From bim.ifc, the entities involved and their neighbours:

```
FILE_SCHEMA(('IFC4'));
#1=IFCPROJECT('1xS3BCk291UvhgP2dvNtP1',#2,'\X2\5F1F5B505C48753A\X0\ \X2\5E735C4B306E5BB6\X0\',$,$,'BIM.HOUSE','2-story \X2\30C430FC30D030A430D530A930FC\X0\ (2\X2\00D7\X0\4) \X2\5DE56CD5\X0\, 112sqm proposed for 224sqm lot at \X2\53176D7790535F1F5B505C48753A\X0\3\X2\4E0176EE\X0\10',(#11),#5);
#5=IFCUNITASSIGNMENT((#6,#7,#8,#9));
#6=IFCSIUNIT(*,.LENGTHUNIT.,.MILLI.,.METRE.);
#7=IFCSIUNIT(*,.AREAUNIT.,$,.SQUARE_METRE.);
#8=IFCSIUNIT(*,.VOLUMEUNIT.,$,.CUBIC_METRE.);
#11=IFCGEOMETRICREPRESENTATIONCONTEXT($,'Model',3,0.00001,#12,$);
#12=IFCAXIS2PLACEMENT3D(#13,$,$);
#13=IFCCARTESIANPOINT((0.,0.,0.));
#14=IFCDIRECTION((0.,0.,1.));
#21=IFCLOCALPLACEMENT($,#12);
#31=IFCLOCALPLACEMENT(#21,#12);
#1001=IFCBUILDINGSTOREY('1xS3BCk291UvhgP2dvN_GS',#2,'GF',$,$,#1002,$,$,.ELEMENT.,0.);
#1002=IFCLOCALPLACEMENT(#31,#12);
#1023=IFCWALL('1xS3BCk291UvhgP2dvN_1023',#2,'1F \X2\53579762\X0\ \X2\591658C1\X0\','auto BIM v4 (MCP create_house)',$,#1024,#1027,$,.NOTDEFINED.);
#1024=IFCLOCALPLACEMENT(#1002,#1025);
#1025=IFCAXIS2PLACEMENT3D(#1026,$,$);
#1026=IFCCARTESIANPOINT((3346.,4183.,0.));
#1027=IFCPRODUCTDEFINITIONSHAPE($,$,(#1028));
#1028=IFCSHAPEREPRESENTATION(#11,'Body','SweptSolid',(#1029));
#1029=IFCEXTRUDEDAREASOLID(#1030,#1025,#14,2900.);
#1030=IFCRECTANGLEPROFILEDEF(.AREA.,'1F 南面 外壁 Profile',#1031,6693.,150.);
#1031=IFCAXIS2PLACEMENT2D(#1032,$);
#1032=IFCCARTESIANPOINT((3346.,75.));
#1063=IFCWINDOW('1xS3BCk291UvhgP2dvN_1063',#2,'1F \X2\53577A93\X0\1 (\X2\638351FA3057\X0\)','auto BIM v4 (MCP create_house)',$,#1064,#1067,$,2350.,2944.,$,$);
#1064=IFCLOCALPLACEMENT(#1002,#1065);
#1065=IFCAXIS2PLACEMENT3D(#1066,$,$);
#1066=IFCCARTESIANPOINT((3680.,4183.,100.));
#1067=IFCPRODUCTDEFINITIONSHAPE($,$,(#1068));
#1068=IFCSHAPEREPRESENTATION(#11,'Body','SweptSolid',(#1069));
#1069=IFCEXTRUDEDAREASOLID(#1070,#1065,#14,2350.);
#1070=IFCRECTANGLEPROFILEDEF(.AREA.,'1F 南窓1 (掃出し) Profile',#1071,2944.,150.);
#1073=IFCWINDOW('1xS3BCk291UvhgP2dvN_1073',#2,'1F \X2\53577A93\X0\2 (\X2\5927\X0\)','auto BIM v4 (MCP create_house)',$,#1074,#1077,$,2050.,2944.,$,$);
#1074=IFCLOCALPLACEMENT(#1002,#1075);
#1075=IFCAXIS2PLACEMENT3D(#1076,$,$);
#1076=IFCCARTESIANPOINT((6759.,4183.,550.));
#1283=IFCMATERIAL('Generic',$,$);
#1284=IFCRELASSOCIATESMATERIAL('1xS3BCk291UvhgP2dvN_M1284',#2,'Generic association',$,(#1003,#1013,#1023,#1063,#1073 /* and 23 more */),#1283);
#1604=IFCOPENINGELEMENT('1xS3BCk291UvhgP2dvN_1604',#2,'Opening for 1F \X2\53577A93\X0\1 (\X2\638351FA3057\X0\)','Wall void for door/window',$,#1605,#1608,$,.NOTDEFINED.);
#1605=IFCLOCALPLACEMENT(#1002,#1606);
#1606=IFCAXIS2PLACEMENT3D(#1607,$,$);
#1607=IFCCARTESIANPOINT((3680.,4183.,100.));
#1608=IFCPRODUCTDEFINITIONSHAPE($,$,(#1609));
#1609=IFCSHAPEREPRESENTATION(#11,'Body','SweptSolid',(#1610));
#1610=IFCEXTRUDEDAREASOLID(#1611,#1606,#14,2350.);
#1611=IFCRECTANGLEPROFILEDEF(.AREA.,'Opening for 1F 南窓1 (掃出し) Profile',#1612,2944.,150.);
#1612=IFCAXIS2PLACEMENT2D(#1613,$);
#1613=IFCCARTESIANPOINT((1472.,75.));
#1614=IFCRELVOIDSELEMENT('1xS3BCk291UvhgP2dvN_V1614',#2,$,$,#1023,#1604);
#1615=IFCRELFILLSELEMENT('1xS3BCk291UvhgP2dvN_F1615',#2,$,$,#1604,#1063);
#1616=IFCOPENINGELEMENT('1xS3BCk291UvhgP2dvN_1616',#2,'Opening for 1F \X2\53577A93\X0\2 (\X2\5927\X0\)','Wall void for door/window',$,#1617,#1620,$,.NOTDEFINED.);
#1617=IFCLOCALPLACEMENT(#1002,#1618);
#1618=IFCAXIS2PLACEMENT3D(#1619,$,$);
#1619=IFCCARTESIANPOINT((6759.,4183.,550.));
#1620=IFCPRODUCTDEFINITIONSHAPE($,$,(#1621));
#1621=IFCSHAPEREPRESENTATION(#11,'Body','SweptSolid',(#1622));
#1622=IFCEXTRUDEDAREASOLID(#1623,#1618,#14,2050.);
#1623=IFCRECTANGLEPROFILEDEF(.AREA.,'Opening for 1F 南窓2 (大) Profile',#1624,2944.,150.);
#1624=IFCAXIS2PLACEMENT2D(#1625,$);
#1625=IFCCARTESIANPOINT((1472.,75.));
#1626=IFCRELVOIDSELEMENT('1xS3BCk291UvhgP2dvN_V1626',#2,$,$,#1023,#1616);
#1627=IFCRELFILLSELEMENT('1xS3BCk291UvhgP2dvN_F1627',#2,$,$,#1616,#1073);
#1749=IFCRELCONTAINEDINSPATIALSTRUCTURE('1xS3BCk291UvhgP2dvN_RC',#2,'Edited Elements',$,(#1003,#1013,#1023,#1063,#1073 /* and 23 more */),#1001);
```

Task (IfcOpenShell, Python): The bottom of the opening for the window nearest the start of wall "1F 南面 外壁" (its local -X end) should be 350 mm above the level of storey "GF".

```python
import numpy as np
import ifcopenshell
import ifcopenshell.api.geometry
import ifcopenshell.geom
import ifcopenshell.util.element
import ifcopenshell.util.placement
import ifcopenshell.util.shape
import ifcopenshell.util.unit

model = ifcopenshell.open("bim.ifc")
unit_scale = ifcopenshell.util.unit.calculate_unit_scale(model)

window = model.by_guid("1xS3BCk291UvhgP2dvN_1063")
opening = window.FillsVoids[0].RelatingOpeningElement
storey = ifcopenshell.util.element.get_container(window, ifc_class="IfcBuildingStorey")
level = ifcopenshell.util.placement.get_local_placement(storey.ObjectPlacement)[2, 3]

# The opening's origin need not be at the sill, so measure its lowest point.
shape = ifcopenshell.geom.create_shape(ifcopenshell.geom.settings(), opening)
bottom = ifcopenshell.util.shape.get_shape_bottom_elevation(shape, shape.geometry) / unit_scale
dz = level + 0.35 / unit_scale - bottom

shift = np.array([0.0, 0.0, dz])
# The window is not placed relative to its opening, so move both.
for product in (opening, window):
    matrix = ifcopenshell.util.placement.get_local_placement(product.ObjectPlacement)
    matrix[:3, 3] += shift
    ifcopenshell.api.geometry.edit_object_placement(model, product=product, matrix=matrix, is_si=False)

print(f"moved by {dz * unit_scale:+.3f} m")

model.write("bim-out.ifc")
```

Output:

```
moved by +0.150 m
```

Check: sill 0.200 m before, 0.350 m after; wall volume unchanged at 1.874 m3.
